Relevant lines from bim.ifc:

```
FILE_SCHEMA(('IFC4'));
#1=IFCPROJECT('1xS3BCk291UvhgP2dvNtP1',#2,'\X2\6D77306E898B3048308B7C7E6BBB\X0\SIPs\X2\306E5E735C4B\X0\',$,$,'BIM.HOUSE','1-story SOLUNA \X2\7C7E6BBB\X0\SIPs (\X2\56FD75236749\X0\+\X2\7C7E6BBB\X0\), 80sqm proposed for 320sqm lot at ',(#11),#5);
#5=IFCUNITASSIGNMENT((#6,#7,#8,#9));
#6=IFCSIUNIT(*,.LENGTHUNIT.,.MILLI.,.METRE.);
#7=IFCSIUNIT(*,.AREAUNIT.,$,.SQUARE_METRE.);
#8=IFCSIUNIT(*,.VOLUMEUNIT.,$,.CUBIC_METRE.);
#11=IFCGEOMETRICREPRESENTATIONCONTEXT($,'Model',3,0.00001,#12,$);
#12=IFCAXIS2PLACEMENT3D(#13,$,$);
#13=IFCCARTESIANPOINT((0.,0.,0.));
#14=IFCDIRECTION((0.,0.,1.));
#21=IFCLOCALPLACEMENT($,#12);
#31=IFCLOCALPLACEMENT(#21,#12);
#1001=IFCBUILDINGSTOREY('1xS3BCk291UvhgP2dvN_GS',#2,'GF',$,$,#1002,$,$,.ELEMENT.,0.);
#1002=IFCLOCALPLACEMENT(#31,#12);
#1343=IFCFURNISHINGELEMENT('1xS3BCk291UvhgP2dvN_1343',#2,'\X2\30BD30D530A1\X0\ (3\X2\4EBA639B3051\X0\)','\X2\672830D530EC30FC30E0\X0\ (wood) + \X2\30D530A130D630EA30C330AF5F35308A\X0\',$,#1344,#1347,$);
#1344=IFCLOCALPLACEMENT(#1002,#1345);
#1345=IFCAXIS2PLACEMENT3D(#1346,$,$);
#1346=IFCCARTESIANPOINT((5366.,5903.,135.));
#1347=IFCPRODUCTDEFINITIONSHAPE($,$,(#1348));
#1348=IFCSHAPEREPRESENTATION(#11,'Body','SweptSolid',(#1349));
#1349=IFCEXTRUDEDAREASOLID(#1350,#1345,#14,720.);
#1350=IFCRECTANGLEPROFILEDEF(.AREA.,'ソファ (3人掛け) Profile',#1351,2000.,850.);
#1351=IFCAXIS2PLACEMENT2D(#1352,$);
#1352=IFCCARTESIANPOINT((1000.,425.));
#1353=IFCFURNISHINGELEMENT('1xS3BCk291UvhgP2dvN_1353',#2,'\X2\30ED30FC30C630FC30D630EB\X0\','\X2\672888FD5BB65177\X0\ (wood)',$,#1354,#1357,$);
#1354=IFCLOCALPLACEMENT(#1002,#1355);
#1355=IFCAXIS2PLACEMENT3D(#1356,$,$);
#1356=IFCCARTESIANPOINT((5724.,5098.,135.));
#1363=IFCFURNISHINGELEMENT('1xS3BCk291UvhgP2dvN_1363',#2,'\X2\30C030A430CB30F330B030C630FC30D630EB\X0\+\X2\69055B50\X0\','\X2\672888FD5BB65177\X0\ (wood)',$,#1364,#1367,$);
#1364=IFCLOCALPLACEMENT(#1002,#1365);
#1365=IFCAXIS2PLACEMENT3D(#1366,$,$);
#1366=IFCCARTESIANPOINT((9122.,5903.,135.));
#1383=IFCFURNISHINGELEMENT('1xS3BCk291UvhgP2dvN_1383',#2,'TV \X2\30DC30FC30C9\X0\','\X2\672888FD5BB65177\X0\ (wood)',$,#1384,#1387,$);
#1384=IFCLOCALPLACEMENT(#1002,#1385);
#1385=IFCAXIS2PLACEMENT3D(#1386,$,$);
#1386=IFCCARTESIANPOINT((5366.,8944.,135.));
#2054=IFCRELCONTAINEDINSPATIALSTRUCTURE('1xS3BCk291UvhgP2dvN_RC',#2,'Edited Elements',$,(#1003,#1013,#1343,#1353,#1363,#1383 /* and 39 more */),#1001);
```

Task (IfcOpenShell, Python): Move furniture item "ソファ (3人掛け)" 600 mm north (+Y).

```python
import ifcopenshell
import ifcopenshell.api.geometry
import ifcopenshell.util.placement
import ifcopenshell.util.unit

model = ifcopenshell.open("bim.ifc")
unit_scale = ifcopenshell.util.unit.calculate_unit_scale(model)

item = model.by_id(1343)
matrix = ifcopenshell.util.placement.get_local_placement(item.ObjectPlacement)
matrix[1, 3] += 0.6 / unit_scale
ifcopenshell.api.geometry.edit_object_placement(model, product=item, matrix=matrix, is_si=False)

print(ifcopenshell.util.placement.get_local_placement(item.ObjectPlacement).round(3) + 0.0)

model.write("bim_rev.ifc")
```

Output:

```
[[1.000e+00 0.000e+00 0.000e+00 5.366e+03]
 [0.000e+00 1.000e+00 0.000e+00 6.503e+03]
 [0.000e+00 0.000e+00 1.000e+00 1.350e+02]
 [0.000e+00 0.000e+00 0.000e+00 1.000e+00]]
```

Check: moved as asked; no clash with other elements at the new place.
